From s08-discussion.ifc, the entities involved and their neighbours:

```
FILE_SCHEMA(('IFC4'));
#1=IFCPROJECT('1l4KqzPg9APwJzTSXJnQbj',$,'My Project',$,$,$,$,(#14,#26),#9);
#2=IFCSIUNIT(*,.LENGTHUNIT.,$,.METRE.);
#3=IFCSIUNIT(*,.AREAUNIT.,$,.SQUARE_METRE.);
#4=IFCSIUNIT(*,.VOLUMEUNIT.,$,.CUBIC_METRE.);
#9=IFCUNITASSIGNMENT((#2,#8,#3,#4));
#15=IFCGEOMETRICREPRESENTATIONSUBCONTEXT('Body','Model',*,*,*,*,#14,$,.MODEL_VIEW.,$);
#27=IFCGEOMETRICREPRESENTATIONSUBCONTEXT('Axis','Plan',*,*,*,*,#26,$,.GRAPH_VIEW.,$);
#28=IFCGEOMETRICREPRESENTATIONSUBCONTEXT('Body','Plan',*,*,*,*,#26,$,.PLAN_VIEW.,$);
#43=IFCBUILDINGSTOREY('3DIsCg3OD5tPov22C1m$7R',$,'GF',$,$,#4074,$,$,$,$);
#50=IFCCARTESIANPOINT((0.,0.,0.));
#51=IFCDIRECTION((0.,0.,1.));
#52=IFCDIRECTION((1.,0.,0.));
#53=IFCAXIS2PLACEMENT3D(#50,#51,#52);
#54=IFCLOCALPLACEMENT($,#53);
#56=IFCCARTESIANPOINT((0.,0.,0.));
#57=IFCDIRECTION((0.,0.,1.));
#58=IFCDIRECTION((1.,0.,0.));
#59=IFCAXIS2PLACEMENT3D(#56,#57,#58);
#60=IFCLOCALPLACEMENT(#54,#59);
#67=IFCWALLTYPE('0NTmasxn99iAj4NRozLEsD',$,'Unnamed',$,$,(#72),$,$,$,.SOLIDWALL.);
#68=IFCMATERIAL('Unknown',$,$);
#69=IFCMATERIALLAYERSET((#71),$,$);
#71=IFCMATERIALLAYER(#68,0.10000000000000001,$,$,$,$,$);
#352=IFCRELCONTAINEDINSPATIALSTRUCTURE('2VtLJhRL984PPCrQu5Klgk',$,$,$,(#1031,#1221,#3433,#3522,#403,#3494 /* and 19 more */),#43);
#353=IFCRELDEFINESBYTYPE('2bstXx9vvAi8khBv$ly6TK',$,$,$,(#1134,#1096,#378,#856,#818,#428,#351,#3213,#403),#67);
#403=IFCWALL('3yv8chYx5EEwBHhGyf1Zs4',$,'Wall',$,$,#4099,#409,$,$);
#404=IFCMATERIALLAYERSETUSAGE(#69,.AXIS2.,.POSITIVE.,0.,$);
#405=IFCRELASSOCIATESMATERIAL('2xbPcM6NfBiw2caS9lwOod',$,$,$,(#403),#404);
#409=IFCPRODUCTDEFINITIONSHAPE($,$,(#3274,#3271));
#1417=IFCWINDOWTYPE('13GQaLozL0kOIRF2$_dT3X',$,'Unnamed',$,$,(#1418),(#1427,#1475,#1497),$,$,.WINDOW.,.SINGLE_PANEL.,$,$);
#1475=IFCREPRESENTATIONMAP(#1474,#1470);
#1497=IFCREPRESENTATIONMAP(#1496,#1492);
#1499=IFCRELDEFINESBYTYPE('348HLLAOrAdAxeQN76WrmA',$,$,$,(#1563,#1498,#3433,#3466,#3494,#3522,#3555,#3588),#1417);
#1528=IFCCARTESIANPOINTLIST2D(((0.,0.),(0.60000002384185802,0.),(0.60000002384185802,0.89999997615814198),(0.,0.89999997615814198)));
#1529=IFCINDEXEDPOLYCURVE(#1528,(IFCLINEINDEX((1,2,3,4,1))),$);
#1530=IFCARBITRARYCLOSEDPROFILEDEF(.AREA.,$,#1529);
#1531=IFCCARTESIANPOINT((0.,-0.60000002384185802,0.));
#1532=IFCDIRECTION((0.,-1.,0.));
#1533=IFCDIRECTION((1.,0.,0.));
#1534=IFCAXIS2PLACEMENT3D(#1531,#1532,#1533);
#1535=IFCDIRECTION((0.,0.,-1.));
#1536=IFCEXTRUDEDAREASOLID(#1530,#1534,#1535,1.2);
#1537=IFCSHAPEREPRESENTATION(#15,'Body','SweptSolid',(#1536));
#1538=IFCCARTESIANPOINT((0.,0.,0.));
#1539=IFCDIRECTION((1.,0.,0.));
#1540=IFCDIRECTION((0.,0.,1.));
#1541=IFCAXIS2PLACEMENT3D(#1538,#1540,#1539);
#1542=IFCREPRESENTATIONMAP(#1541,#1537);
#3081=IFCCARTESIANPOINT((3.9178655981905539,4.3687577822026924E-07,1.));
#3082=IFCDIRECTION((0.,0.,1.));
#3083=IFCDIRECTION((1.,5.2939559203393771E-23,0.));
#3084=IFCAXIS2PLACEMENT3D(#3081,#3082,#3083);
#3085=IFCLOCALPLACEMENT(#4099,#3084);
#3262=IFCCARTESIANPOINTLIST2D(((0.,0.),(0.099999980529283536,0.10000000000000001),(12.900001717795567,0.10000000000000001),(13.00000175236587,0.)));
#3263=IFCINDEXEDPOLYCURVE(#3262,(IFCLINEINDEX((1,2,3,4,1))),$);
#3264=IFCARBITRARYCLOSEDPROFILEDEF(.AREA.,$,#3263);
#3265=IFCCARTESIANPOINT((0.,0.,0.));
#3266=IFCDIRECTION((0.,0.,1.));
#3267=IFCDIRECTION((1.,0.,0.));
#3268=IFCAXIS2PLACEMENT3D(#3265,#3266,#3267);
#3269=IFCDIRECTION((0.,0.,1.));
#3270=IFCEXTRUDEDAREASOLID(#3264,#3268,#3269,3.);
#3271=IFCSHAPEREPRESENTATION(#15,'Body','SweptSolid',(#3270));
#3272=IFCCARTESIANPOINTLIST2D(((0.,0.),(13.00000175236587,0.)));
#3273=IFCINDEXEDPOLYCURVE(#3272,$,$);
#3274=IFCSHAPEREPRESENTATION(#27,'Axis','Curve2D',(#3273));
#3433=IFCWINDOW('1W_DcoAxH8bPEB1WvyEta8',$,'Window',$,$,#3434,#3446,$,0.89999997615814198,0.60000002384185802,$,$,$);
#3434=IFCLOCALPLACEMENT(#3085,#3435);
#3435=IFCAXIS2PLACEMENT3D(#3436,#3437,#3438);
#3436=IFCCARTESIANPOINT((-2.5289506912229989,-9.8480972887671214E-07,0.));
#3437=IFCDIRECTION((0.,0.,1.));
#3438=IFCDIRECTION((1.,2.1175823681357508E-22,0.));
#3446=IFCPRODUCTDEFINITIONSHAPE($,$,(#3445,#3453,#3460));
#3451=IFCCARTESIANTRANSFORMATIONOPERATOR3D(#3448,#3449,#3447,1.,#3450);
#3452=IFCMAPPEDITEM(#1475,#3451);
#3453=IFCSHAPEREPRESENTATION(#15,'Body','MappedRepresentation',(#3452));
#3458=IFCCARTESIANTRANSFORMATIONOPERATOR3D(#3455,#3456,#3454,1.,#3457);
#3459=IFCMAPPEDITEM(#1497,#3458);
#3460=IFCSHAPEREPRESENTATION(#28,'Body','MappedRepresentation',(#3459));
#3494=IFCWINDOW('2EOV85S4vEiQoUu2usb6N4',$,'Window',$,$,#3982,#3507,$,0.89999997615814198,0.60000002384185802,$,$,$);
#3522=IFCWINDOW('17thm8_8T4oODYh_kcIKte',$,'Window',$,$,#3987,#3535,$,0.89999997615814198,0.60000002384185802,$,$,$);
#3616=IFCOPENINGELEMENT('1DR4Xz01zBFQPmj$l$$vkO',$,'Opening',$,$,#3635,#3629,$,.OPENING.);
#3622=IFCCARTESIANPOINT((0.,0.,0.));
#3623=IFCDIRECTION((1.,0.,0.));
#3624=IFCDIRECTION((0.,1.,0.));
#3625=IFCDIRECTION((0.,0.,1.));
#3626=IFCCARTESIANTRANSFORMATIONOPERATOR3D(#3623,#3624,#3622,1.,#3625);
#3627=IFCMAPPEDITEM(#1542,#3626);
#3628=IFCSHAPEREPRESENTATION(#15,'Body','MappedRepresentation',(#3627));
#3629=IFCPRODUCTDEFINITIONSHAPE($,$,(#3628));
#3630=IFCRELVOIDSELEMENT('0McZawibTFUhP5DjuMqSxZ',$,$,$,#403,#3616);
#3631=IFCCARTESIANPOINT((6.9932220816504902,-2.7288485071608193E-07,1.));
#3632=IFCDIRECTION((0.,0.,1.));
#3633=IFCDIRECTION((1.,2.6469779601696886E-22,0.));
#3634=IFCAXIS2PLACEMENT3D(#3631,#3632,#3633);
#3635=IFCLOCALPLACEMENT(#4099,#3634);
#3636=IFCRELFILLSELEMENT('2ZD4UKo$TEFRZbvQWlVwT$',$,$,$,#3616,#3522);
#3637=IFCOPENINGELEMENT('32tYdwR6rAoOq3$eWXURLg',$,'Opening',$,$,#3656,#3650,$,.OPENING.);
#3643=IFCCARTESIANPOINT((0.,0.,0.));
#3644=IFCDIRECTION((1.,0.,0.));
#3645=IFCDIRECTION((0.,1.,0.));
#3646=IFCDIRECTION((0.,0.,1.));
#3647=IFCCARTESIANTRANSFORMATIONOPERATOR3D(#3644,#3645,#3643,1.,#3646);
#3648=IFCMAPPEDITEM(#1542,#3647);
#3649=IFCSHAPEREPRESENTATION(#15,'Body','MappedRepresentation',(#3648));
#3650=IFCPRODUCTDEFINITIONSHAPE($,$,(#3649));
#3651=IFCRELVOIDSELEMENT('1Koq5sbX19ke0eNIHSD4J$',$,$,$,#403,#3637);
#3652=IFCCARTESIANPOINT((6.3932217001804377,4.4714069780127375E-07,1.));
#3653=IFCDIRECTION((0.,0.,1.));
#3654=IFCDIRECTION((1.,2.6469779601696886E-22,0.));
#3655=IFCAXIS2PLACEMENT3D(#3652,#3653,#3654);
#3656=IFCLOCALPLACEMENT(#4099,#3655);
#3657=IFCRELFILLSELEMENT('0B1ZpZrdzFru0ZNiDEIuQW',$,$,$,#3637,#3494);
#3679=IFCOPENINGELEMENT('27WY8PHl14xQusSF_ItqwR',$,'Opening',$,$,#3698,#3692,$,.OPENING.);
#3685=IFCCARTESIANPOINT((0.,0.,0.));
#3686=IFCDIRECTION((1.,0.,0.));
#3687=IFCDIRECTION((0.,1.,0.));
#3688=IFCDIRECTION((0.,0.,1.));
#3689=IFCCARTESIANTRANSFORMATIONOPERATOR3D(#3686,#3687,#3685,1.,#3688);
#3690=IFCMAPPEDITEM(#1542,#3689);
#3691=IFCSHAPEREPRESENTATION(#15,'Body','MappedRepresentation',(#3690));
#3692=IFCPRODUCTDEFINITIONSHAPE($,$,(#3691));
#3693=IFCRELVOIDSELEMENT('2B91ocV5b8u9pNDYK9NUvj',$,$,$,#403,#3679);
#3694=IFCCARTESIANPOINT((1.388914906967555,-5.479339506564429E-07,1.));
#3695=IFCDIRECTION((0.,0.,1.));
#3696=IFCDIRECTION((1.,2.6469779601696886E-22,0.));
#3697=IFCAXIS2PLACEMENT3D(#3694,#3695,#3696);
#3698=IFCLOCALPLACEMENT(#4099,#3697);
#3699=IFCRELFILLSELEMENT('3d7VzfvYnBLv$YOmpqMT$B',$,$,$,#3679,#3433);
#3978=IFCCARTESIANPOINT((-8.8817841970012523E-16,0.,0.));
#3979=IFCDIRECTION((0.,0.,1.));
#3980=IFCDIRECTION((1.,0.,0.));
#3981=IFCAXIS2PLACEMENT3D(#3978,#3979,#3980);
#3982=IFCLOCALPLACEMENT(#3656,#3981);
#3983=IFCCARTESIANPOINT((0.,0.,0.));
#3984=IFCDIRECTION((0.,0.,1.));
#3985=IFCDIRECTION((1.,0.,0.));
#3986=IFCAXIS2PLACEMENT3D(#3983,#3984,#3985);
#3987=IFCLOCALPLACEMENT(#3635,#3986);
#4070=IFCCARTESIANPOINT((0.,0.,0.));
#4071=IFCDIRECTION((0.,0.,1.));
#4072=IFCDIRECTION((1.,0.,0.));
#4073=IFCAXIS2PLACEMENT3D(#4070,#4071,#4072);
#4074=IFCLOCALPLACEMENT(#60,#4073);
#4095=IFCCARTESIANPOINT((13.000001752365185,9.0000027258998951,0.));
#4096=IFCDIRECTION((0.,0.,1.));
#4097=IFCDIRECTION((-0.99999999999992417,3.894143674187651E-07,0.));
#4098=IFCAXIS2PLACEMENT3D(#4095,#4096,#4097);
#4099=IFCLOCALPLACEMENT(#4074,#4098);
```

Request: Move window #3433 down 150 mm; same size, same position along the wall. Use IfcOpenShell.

```python
import numpy as np
import ifcopenshell
import ifcopenshell.api.geometry
import ifcopenshell.util.placement
import ifcopenshell.util.unit

model = ifcopenshell.open("s08-discussion.ifc")
unit_scale = ifcopenshell.util.unit.calculate_unit_scale(model)

window = model.by_guid("1W_DcoAxH8bPEB1WvyEta8")
opening = window.FillsVoids[0].RelatingOpeningElement
dz = -0.15 / unit_scale

shift = np.array([0.0, 0.0, dz])
# The window is not placed relative to its opening, so move both.
for product in (opening, window):
    matrix = ifcopenshell.util.placement.get_local_placement(product.ObjectPlacement)
    matrix[:3, 3] += shift
    ifcopenshell.api.geometry.edit_object_placement(model, product=product, matrix=matrix, is_si=False)

print(f"moved by {dz * unit_scale:+.3f} m")

model.write("s08-discussion_rev.ifc")
```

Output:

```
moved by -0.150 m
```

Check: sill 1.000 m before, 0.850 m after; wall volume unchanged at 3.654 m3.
